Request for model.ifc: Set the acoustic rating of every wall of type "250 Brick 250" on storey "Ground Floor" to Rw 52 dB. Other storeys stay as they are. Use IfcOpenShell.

First a look at what the model holds.

```python
import ifcopenshell
import ifcopenshell.util.element

model = ifcopenshell.open("model.ifc")
print(model.schema)
storey = next(s for s in model.by_type("IfcBuildingStorey") if s.Name == "Ground Floor")
walls = [e for e in ifcopenshell.util.element.get_decomposition(storey) if e.is_a("IfcWall")]
seen = {}
for e in walls:
    element_type = ifcopenshell.util.element.get_type(e)
    key = (element_type.Name if element_type != e and element_type else None, ifcopenshell.util.element.get_pset(e, "Pset_WallCommon", "AcousticRating"))
    seen[key] = seen.get(key, 0) + 1
for (name, value), count in sorted(seen.items(), key=str):
    print(count, "x", name, "|", value)
```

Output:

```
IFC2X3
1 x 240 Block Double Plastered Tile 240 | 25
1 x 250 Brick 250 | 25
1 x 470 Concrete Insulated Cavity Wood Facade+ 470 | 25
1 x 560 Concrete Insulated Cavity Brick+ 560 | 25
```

```python
import ifcopenshell
import ifcopenshell.api.pset
import ifcopenshell.util.element

model = ifcopenshell.open("model.ifc")

storey = next(s for s in model.by_type("IfcBuildingStorey") if s.Name == "Ground Floor")
walls = [e for e in ifcopenshell.util.element.get_decomposition(storey) if e.is_a("IfcWall")]

count = 0
for e in walls:
    element_type = ifcopenshell.util.element.get_type(e)
    if element_type in (None, e) or element_type.Name != "250 Brick 250":
        continue
    # add_pset returns the element's existing set when there is one.
    pset = ifcopenshell.api.pset.add_pset(model, product=e, name="Pset_WallCommon")
    ifcopenshell.api.pset.edit_pset(model, pset=pset, properties={"AcousticRating": "Rw 52 dB"})
    count += 1

print(count, "walls updated")

model.write("model_edited.ifc")
```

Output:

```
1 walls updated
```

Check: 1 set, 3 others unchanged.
